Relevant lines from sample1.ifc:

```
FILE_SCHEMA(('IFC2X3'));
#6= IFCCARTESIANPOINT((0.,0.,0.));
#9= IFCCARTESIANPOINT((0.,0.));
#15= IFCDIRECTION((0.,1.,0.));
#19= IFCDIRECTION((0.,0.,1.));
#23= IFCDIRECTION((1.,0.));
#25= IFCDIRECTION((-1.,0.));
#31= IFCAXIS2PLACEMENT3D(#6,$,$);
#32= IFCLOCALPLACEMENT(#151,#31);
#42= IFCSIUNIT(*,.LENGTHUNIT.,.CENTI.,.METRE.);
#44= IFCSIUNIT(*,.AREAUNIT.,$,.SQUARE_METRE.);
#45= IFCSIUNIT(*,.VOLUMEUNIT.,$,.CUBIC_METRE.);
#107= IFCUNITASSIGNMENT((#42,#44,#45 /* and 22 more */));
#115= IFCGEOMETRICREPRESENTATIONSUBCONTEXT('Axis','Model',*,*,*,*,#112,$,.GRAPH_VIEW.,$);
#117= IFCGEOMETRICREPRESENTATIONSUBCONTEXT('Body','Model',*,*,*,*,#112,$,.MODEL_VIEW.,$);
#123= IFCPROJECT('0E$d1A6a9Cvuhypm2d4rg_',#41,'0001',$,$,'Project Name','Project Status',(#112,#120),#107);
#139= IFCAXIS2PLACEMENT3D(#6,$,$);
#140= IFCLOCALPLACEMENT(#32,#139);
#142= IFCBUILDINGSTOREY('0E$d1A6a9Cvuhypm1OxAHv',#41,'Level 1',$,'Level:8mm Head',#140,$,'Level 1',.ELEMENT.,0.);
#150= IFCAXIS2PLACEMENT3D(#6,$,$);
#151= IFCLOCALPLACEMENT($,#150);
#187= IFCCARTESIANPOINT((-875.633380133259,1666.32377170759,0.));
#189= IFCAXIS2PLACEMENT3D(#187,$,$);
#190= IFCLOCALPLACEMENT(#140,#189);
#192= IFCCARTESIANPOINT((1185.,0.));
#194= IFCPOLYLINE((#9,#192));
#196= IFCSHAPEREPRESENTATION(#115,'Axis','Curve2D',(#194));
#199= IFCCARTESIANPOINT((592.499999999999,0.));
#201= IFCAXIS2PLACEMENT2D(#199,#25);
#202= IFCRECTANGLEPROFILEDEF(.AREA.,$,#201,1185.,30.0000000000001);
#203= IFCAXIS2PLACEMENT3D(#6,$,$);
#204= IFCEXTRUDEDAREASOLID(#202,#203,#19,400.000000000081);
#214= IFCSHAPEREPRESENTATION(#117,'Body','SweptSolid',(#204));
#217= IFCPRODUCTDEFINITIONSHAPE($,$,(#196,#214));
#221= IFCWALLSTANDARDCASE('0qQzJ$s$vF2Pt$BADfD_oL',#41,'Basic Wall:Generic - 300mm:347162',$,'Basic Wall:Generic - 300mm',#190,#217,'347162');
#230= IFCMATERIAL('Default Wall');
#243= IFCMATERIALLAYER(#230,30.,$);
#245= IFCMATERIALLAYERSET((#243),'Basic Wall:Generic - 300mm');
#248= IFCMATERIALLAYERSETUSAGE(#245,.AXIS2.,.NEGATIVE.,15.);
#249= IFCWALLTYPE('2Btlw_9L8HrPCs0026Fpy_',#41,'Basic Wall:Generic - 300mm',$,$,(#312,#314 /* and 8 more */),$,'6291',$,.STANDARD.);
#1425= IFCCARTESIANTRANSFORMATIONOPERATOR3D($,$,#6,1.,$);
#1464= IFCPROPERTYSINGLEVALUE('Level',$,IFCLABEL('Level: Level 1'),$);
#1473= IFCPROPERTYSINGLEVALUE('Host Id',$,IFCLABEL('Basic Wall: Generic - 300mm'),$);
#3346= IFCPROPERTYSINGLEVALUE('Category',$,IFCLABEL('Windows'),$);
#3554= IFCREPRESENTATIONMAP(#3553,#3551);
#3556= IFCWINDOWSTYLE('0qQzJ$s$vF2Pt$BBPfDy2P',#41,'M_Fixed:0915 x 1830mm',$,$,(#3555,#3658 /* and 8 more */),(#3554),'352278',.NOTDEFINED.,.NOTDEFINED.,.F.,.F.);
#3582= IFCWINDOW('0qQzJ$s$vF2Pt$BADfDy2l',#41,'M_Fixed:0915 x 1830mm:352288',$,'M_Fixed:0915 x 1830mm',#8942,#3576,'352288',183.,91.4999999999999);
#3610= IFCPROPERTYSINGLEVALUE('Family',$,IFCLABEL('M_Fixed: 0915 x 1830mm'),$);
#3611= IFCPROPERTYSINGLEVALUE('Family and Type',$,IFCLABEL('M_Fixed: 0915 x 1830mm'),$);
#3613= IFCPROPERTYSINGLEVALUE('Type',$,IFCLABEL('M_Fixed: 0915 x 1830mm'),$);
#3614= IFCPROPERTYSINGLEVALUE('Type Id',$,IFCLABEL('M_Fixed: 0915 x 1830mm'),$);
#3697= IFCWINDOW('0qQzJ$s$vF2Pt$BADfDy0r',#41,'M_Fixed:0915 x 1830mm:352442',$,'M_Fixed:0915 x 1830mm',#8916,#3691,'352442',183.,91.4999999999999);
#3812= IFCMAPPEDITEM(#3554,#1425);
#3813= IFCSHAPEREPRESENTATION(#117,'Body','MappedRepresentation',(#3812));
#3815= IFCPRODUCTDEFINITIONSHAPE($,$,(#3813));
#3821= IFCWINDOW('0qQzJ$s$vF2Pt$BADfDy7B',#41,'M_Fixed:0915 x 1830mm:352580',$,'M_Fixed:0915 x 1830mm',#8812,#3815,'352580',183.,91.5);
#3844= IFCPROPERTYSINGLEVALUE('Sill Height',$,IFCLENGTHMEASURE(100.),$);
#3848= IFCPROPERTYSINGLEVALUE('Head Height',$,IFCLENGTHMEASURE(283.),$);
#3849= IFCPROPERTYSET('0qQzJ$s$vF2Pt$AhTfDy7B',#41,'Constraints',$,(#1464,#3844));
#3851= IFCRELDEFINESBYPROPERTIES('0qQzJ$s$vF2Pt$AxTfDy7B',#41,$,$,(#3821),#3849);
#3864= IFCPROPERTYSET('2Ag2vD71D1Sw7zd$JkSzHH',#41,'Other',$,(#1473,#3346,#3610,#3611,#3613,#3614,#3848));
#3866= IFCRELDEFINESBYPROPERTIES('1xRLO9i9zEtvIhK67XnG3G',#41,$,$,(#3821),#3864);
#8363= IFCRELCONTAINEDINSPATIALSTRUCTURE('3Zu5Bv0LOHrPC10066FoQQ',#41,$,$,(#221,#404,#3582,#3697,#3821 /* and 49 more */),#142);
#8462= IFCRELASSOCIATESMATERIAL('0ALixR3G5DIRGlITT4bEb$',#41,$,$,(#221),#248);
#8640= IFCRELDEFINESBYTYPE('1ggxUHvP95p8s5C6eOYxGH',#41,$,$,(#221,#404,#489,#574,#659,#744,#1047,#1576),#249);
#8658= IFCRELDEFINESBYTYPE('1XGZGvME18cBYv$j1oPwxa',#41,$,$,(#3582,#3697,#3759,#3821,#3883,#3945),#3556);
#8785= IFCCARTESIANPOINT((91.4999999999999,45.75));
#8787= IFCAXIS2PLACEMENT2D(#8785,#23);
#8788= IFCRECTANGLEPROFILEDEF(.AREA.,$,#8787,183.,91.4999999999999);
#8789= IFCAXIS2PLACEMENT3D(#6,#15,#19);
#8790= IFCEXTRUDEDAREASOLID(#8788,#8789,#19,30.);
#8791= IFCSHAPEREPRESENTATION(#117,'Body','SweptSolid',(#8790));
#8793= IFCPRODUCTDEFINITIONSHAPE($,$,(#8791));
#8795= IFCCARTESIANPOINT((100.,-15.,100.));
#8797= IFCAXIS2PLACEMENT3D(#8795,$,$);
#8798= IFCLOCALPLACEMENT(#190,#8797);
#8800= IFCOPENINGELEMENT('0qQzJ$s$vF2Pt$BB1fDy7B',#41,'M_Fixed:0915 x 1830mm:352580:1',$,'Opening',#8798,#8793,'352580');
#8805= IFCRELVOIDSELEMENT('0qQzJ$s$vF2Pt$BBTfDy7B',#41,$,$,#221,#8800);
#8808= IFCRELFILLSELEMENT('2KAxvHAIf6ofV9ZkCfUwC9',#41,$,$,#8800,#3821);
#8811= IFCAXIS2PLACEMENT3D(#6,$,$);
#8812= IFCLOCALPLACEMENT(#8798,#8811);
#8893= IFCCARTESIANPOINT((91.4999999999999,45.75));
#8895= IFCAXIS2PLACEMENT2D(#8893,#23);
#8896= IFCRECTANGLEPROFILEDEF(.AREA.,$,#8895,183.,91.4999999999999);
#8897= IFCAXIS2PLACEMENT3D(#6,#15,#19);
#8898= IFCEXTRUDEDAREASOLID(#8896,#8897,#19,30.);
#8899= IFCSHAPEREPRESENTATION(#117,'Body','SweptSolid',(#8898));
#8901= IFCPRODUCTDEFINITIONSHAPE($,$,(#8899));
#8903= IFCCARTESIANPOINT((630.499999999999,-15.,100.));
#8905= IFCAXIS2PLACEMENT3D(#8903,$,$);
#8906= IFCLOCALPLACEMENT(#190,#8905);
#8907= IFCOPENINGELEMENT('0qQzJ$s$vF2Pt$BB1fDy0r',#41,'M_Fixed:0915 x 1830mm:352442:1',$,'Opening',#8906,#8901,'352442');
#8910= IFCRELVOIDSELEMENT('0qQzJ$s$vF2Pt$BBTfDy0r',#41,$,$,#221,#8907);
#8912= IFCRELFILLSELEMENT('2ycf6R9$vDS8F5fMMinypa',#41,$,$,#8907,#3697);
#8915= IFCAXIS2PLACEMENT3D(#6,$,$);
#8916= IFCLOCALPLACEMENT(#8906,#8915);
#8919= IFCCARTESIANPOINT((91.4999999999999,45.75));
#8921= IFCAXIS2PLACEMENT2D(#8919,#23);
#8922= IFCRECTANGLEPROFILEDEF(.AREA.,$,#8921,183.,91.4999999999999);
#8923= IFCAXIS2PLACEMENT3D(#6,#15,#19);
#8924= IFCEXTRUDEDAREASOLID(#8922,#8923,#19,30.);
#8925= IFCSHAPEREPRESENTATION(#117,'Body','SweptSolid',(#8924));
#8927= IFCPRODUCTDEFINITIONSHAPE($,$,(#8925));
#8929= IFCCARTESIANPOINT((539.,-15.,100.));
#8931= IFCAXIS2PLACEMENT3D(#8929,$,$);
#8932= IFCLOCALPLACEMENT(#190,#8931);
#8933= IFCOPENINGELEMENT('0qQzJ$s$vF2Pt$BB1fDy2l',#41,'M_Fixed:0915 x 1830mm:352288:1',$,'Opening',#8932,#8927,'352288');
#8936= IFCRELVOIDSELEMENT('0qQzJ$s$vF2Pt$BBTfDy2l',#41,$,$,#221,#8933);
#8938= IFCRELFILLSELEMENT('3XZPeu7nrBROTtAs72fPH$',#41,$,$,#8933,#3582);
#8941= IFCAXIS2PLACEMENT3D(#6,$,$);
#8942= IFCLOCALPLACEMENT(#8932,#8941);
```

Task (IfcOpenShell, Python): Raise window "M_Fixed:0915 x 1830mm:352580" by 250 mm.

```python
import numpy as np
import ifcopenshell
import ifcopenshell.api.geometry
import ifcopenshell.api.pset
import ifcopenshell.util.element
import ifcopenshell.util.placement
import ifcopenshell.util.unit

model = ifcopenshell.open("sample1.ifc")
unit_scale = ifcopenshell.util.unit.calculate_unit_scale(model)

window = model.by_id(3821)
opening = window.FillsVoids[0].RelatingOpeningElement
dz = 0.25 / unit_scale

shift = np.array([0.0, 0.0, dz])
# The window is placed relative to its opening, so it follows when the opening moves.
matrix = ifcopenshell.util.placement.get_local_placement(opening.ObjectPlacement)
matrix[:3, 3] += shift
ifcopenshell.api.geometry.edit_object_placement(
    model, product=opening, matrix=matrix, is_si=False, should_transform_children=True
)

# Keep the stored heights in step.
pset = model.by_id(ifcopenshell.util.element.get_pset(window, "Constraints", should_inherit=False)["id"])
ifcopenshell.api.pset.edit_pset(model, pset=pset, properties={
    "Sill Height": model.create_entity("IfcLengthMeasure", ifcopenshell.util.element.get_pset(window, "Constraints", "Sill Height") + dz),
})
pset = model.by_id(ifcopenshell.util.element.get_pset(window, "Other", should_inherit=False)["id"])
ifcopenshell.api.pset.edit_pset(model, pset=pset, properties={
    "Head Height": model.create_entity("IfcLengthMeasure", ifcopenshell.util.element.get_pset(window, "Other", "Head Height") + dz),
})

print(f"moved by {dz * unit_scale:+.3f} m")

model.write("sample1_v2.ifc")
```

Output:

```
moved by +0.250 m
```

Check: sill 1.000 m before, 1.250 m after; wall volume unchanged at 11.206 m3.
